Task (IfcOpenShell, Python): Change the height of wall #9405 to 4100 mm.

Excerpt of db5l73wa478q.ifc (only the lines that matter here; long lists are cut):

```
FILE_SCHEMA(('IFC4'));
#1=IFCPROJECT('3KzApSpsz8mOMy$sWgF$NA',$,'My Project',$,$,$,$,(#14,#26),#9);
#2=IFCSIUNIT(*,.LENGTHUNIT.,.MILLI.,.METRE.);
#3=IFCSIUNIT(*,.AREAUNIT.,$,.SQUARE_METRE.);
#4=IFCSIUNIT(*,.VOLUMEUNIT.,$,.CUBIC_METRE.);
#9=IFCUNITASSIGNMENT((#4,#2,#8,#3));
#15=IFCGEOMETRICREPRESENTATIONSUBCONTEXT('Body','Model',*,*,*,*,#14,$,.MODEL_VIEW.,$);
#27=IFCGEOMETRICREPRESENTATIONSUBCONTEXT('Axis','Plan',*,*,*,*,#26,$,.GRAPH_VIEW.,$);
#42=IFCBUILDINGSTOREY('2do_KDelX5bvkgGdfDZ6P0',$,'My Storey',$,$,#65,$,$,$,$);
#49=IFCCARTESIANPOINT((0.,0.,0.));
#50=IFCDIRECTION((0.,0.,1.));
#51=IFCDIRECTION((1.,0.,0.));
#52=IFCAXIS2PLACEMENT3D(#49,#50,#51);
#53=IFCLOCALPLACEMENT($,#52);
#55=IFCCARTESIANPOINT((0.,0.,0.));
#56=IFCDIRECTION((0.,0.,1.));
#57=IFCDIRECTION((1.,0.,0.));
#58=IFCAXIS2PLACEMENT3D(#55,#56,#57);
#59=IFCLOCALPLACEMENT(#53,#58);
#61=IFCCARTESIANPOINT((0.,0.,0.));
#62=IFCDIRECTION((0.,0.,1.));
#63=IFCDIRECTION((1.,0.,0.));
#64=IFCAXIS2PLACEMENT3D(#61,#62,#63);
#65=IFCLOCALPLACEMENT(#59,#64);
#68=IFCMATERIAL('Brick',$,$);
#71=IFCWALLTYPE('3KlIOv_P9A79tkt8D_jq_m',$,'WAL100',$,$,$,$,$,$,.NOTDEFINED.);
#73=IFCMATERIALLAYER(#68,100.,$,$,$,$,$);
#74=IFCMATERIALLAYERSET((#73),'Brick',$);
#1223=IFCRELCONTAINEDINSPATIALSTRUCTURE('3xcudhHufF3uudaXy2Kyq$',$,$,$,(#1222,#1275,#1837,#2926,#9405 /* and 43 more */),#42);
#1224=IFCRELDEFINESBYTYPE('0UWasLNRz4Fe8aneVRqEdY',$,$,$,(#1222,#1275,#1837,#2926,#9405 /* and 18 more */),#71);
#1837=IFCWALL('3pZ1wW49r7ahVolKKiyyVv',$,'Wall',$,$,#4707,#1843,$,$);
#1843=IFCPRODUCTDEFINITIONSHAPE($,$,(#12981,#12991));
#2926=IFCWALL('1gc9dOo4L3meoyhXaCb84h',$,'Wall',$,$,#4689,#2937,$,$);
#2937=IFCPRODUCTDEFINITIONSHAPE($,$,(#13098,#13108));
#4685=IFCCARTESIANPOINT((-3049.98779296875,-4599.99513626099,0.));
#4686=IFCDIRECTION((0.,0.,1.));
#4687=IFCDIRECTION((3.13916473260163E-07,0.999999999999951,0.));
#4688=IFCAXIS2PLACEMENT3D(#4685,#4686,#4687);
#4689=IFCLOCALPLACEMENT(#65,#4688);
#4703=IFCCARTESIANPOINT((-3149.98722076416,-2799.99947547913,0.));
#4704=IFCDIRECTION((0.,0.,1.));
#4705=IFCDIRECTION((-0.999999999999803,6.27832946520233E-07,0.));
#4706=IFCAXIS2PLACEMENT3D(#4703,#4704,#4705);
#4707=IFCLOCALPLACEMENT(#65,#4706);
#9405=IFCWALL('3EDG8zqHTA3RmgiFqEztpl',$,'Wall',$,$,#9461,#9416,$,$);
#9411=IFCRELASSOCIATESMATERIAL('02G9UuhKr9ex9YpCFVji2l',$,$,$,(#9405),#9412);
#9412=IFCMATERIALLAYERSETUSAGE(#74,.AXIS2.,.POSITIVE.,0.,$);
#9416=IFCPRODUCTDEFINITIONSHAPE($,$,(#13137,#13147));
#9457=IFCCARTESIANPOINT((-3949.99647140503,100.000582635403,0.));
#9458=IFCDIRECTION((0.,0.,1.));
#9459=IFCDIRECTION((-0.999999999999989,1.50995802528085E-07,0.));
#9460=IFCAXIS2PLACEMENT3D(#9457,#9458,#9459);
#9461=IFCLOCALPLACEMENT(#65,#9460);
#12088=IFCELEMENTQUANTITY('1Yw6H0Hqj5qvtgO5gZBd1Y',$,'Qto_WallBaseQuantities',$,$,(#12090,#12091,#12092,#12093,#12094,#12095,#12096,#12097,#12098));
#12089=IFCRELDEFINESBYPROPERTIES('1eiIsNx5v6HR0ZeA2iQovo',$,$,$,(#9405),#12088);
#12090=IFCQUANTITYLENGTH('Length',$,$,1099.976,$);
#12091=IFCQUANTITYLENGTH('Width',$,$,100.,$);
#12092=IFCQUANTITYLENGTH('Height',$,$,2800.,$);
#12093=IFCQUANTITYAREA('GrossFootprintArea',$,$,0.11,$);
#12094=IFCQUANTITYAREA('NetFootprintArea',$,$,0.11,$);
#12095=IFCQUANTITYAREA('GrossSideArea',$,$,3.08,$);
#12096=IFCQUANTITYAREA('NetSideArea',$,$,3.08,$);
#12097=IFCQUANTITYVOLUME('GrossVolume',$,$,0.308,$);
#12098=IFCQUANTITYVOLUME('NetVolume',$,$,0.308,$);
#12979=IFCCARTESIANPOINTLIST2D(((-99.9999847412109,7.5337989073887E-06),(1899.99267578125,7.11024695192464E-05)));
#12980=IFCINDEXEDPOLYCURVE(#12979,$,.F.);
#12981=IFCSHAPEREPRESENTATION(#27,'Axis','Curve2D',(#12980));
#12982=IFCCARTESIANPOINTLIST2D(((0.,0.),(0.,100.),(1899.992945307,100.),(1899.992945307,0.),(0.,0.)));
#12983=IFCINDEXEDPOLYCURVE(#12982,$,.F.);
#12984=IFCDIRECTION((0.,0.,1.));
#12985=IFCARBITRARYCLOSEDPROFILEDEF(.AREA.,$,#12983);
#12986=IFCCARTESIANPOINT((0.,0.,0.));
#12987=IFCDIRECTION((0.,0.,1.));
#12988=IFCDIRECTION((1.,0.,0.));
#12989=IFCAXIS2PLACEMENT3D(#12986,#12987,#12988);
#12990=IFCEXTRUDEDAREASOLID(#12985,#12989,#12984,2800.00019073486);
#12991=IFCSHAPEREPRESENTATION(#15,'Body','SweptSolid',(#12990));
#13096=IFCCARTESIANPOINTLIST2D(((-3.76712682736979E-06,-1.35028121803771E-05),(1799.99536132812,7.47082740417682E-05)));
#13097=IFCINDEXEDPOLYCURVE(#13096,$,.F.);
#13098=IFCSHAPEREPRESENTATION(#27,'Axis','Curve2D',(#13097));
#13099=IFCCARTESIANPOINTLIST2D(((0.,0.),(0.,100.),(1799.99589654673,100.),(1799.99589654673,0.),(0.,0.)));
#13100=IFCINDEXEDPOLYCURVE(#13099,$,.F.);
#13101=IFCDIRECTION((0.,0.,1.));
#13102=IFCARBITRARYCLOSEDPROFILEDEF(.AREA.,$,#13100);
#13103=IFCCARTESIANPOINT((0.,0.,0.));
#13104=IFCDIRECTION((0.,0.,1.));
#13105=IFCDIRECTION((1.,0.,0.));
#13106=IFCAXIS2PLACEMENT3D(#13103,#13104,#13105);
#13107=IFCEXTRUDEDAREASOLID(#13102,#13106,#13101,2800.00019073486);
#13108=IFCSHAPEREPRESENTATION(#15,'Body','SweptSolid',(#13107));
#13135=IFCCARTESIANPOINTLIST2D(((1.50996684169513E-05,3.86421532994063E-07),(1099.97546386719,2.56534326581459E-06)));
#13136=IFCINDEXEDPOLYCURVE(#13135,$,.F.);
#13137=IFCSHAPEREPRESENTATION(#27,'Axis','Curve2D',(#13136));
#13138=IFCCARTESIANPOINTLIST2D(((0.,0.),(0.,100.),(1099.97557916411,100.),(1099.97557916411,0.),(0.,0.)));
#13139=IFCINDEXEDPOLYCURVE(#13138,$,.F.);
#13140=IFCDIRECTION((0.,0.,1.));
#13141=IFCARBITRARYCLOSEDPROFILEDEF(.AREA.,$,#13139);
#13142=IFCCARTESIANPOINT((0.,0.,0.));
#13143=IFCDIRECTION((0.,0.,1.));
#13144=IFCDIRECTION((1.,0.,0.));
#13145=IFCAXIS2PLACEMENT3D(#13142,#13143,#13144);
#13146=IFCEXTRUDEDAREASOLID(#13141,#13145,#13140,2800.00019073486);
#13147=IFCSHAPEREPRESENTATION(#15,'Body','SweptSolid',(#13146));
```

```python
import ifcopenshell
import ifcopenshell.api.pset
import ifcopenshell.geom
import ifcopenshell.util.element
import ifcopenshell.util.representation
import ifcopenshell.util.shape
import ifcopenshell.util.unit

model = ifcopenshell.open("db5l73wa478q.ifc")
unit_scale = ifcopenshell.util.unit.calculate_unit_scale(model)
area_scale = ifcopenshell.util.unit.calculate_unit_scale(model, "AREAUNIT")
volume_scale = ifcopenshell.util.unit.calculate_unit_scale(model, "VOLUMEUNIT")
settings = ifcopenshell.geom.settings()


def volume(element):
    """Net volume in cubic metres, openings subtracted."""
    shape = ifcopenshell.geom.create_shape(settings, element)
    return ifcopenshell.util.shape.get_volume(shape.geometry)


wall = model.by_guid("3EDG8zqHTA3RmgiFqEztpl")
before = volume(wall)

body = ifcopenshell.util.representation.get_representation(wall, "Model", "Body")
solid = body.Items[0]
old_height = solid.Depth
solid.Depth = 4.1 / unit_scale
after = volume(wall)
thickness = 0.1  # wall thickness in metres

# Update the stored height, areas and volumes.
qto = model.by_id(ifcopenshell.util.element.get_pset(wall, "Qto_WallBaseQuantities", should_inherit=False)["id"])
ifcopenshell.api.pset.edit_qto(model, qto=qto, properties={
    "Height": solid.Depth,
    "GrossSideArea": ifcopenshell.util.element.get_pset(wall, "Qto_WallBaseQuantities", "GrossSideArea") * solid.Depth / old_height,
    "NetSideArea": after / thickness / area_scale,
    "GrossVolume": ifcopenshell.util.element.get_pset(wall, "Qto_WallBaseQuantities", "GrossVolume") * solid.Depth / old_height,
    "NetVolume": after / volume_scale,
})

print(f"height {old_height:g} -> {solid.Depth:g}, volume {before:.3f} -> {after:.3f} m3")

model.write("db5l73wa478q_edited.ifc")
```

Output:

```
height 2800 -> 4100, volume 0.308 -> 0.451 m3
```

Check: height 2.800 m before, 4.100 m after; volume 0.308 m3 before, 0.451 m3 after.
